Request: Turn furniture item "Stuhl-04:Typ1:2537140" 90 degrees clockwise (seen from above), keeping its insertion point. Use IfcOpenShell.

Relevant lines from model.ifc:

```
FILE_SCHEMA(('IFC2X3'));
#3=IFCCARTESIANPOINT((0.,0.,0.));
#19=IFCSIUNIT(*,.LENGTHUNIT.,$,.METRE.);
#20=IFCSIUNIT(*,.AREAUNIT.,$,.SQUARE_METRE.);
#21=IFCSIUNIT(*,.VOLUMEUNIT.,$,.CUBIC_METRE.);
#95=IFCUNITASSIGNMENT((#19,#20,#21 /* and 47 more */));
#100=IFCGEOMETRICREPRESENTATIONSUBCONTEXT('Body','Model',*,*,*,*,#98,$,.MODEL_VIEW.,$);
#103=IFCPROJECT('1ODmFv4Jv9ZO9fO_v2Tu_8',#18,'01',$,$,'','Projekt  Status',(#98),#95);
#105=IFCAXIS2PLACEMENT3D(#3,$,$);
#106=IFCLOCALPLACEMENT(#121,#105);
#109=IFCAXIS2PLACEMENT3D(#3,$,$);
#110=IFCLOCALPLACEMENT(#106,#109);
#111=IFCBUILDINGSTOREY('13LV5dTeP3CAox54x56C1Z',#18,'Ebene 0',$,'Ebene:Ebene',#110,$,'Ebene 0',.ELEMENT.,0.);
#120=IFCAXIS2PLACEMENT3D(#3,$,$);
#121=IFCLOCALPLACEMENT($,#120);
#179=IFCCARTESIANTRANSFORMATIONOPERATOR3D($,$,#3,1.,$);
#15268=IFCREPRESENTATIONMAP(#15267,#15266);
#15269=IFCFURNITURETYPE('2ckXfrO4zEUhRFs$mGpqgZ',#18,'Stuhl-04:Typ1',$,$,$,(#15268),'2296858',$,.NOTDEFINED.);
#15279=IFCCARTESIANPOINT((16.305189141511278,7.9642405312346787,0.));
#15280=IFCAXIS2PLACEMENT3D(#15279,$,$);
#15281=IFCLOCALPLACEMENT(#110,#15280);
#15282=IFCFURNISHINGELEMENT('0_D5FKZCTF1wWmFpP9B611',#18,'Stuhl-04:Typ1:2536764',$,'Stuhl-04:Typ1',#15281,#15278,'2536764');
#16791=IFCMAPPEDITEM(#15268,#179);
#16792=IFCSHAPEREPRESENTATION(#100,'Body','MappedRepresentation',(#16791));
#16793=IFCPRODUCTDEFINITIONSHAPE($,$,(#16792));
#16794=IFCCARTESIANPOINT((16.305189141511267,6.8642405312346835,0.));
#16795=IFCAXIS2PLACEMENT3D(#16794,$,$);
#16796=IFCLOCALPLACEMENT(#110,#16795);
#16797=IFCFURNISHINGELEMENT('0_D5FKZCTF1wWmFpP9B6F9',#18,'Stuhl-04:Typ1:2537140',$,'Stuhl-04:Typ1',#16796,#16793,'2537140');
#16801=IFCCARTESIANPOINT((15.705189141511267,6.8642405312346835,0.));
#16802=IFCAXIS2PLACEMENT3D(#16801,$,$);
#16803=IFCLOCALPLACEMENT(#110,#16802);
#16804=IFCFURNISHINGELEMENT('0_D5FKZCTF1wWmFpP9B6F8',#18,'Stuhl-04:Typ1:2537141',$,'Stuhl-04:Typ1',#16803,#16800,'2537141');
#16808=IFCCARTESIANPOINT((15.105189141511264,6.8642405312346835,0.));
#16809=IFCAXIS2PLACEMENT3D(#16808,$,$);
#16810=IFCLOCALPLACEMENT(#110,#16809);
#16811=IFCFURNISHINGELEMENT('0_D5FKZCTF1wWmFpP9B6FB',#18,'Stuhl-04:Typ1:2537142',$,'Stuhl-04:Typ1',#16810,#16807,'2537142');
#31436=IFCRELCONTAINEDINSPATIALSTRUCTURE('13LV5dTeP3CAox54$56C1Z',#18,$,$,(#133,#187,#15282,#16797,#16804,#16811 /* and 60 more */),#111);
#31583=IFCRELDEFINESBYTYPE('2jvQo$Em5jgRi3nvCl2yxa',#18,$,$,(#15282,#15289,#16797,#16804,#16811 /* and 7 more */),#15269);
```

```python
import ifcopenshell
import ifcopenshell.api.geometry
import ifcopenshell.util.placement

model = ifcopenshell.open("model.ifc")

item = model.by_guid("0_D5FKZCTF1wWmFpP9B6F9")
matrix = ifcopenshell.util.placement.get_local_placement(item.ObjectPlacement)
matrix = matrix @ ifcopenshell.util.placement.rotation(-90, "Z")
ifcopenshell.api.geometry.edit_object_placement(model, product=item, matrix=matrix, is_si=False)

print(ifcopenshell.util.placement.get_local_placement(item.ObjectPlacement).round(3) + 0.0)

model.write("model-out.ifc")
```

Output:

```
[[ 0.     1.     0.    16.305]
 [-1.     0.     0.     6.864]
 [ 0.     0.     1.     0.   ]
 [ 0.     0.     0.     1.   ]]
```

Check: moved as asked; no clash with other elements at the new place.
